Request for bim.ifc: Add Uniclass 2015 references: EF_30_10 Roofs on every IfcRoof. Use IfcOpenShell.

First a look at what the model holds.

```python
import ifcopenshell

model = ifcopenshell.open("bim.ifc")
print(model.schema)
print("classifications:", [c.Name for c in model.by_type("IfcClassification")])
for ifc_class in ("IfcDoor", "IfcRoof", "IfcStair", "IfcWall", "IfcWindow"):
    print(ifc_class, len(model.by_type(ifc_class)))
```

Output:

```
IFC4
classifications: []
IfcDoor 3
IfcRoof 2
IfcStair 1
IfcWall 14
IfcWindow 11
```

```python
import ifcopenshell
import ifcopenshell.api.classification

model = ifcopenshell.open("bim.ifc")

system = ifcopenshell.api.classification.add_classification(model, classification="Uniclass 2015")

codes = {
    "IfcRoof": ("EF_30_10", "Roofs"),
}
for ifc_class, (code, name) in codes.items():
    products = model.by_type(ifc_class)
    ifcopenshell.api.classification.add_reference(
        model, products=products, classification=system, identification=code, name=name
    )
    print(code, len(products))

model.write("bim_edited.ifc")
```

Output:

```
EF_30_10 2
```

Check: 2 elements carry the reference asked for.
